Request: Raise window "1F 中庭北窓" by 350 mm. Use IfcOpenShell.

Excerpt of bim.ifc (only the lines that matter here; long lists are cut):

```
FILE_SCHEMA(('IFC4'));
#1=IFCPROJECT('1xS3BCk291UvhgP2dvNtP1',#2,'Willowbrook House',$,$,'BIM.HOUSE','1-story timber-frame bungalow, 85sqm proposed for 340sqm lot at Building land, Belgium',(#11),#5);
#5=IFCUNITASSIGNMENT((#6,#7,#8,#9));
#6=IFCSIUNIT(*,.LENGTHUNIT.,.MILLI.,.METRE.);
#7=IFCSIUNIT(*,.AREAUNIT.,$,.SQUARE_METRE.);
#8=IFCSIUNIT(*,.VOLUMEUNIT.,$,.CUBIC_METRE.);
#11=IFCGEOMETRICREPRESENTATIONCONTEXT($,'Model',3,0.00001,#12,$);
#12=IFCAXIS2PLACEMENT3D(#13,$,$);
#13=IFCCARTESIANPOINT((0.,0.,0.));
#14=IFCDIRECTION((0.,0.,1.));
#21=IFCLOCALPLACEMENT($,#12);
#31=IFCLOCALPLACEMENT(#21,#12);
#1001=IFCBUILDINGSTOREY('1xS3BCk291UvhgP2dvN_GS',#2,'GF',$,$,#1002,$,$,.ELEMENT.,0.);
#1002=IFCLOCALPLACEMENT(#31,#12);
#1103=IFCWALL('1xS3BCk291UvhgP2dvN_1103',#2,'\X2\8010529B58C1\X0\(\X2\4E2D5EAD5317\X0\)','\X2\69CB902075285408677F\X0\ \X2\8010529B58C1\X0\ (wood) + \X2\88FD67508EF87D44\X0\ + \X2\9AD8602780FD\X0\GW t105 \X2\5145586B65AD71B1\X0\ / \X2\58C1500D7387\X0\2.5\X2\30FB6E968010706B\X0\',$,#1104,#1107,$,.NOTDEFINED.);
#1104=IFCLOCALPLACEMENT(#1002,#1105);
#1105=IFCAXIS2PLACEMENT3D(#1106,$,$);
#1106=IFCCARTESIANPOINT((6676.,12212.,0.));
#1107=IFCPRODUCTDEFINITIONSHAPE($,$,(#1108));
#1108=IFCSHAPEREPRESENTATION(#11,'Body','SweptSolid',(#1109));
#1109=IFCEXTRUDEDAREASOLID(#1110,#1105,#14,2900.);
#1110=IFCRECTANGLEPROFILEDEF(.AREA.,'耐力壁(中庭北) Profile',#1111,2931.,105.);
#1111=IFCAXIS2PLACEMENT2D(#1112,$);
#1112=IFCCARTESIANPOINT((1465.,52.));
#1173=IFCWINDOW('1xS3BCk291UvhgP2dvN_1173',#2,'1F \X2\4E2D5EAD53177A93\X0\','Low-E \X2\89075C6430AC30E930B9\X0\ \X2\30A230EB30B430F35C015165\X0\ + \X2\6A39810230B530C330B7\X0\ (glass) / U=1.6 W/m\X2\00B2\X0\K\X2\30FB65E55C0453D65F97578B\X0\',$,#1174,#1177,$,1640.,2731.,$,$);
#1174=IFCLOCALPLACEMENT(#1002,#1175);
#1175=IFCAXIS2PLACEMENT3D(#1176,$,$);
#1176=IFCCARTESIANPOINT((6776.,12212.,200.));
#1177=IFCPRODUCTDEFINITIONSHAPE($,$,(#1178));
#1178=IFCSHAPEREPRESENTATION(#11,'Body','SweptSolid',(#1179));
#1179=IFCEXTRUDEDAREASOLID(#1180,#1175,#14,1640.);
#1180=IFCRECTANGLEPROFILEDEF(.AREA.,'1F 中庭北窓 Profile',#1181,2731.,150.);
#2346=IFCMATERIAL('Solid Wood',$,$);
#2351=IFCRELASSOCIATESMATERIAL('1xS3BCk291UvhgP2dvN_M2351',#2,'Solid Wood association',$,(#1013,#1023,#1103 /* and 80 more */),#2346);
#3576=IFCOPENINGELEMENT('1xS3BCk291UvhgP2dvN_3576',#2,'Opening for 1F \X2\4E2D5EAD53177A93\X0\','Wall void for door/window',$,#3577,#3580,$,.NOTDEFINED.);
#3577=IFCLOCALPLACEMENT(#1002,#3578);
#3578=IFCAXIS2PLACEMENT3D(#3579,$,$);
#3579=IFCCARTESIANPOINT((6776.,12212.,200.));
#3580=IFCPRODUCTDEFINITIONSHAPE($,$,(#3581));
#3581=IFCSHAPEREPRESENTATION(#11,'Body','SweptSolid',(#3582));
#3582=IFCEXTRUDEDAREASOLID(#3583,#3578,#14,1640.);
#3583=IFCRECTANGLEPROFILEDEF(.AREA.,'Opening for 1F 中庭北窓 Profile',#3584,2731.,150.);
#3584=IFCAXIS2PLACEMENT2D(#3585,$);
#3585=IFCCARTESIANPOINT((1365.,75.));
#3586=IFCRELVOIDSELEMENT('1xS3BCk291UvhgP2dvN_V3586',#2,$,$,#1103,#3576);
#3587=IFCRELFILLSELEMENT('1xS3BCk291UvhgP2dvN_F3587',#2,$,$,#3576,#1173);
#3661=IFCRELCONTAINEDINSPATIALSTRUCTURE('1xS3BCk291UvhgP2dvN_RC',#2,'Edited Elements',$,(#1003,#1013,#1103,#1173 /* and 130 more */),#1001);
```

```python
import numpy as np
import ifcopenshell
import ifcopenshell.api.geometry
import ifcopenshell.util.placement
import ifcopenshell.util.unit

model = ifcopenshell.open("bim.ifc")
unit_scale = ifcopenshell.util.unit.calculate_unit_scale(model)

window = model.by_guid("1xS3BCk291UvhgP2dvN_1173")
opening = window.FillsVoids[0].RelatingOpeningElement
dz = 350.0

shift = np.array([0.0, 0.0, dz])
# The window is not placed relative to its opening, so move both.
for product in (opening, window):
    matrix = ifcopenshell.util.placement.get_local_placement(product.ObjectPlacement)
    matrix[:3, 3] += shift
    ifcopenshell.api.geometry.edit_object_placement(model, product=product, matrix=matrix, is_si=False)

print(f"moved by {dz * unit_scale:+.3f} m")

model.write("bim_updated.ifc")
```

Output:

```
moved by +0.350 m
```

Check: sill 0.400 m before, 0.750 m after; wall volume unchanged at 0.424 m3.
